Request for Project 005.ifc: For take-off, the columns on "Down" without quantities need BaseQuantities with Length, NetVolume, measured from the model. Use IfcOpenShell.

First a look at what the model holds.

```python
import ifcopenshell
import ifcopenshell.util.element
import ifcopenshell.util.unit

model = ifcopenshell.open("Project 005.ifc")
print(model.schema)
for unit_type in ("LENGTHUNIT", "AREAUNIT", "VOLUMEUNIT"):
    print(unit_type, ifcopenshell.util.unit.calculate_unit_scale(model, unit_type))
storey = next(s for s in model.by_type("IfcBuildingStorey") if s.Name == "Down")
columns = [e for e in ifcopenshell.util.element.get_decomposition(storey) if e.is_a("IfcColumn")]
for e in sorted(columns, key=lambda e: e.id()):
    print(e.id(), e.is_a(), e.Name, list(ifcopenshell.util.element.get_psets(e, qtos_only=True)), sep=" | ")
```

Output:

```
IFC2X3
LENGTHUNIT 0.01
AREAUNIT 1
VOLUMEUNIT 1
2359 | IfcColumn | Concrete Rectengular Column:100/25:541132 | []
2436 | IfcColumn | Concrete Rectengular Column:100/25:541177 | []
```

```python
import ifcopenshell
import ifcopenshell.api.pset
import ifcopenshell.geom
import ifcopenshell.util.element
import ifcopenshell.util.shape
import ifcopenshell.util.unit

model = ifcopenshell.open("Project 005.ifc")
unit_scale = ifcopenshell.util.unit.calculate_unit_scale(model)
volume_scale = ifcopenshell.util.unit.calculate_unit_scale(model, "VOLUMEUNIT")
settings = ifcopenshell.geom.settings()

storey = next(s for s in model.by_type("IfcBuildingStorey") if s.Name == "Down")
columns = [e for e in ifcopenshell.util.element.get_decomposition(storey) if e.is_a("IfcColumn")]

for e in sorted(columns, key=lambda e: e.id()):
    if ifcopenshell.util.element.get_psets(e, qtos_only=True, should_inherit=False):
        continue
    # Geometry comes back in metres, in the element's own axes.
    shape = ifcopenshell.geom.create_shape(settings, e)
    values = {
        "Length": ifcopenshell.util.shape.get_z(shape.geometry) / unit_scale,
        "NetVolume": ifcopenshell.util.shape.get_volume(shape.geometry) / volume_scale,
    }
    qto = ifcopenshell.api.pset.add_qto(model, product=e, name="BaseQuantities")
    ifcopenshell.api.pset.edit_qto(model, qto=qto, properties=values)
    print(e.id(), {k: round(v, 3) for k, v in values.items()})

model.write("Project 005_edited.ifc")
```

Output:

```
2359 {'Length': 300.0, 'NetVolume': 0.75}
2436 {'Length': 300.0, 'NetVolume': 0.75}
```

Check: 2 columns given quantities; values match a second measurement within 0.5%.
